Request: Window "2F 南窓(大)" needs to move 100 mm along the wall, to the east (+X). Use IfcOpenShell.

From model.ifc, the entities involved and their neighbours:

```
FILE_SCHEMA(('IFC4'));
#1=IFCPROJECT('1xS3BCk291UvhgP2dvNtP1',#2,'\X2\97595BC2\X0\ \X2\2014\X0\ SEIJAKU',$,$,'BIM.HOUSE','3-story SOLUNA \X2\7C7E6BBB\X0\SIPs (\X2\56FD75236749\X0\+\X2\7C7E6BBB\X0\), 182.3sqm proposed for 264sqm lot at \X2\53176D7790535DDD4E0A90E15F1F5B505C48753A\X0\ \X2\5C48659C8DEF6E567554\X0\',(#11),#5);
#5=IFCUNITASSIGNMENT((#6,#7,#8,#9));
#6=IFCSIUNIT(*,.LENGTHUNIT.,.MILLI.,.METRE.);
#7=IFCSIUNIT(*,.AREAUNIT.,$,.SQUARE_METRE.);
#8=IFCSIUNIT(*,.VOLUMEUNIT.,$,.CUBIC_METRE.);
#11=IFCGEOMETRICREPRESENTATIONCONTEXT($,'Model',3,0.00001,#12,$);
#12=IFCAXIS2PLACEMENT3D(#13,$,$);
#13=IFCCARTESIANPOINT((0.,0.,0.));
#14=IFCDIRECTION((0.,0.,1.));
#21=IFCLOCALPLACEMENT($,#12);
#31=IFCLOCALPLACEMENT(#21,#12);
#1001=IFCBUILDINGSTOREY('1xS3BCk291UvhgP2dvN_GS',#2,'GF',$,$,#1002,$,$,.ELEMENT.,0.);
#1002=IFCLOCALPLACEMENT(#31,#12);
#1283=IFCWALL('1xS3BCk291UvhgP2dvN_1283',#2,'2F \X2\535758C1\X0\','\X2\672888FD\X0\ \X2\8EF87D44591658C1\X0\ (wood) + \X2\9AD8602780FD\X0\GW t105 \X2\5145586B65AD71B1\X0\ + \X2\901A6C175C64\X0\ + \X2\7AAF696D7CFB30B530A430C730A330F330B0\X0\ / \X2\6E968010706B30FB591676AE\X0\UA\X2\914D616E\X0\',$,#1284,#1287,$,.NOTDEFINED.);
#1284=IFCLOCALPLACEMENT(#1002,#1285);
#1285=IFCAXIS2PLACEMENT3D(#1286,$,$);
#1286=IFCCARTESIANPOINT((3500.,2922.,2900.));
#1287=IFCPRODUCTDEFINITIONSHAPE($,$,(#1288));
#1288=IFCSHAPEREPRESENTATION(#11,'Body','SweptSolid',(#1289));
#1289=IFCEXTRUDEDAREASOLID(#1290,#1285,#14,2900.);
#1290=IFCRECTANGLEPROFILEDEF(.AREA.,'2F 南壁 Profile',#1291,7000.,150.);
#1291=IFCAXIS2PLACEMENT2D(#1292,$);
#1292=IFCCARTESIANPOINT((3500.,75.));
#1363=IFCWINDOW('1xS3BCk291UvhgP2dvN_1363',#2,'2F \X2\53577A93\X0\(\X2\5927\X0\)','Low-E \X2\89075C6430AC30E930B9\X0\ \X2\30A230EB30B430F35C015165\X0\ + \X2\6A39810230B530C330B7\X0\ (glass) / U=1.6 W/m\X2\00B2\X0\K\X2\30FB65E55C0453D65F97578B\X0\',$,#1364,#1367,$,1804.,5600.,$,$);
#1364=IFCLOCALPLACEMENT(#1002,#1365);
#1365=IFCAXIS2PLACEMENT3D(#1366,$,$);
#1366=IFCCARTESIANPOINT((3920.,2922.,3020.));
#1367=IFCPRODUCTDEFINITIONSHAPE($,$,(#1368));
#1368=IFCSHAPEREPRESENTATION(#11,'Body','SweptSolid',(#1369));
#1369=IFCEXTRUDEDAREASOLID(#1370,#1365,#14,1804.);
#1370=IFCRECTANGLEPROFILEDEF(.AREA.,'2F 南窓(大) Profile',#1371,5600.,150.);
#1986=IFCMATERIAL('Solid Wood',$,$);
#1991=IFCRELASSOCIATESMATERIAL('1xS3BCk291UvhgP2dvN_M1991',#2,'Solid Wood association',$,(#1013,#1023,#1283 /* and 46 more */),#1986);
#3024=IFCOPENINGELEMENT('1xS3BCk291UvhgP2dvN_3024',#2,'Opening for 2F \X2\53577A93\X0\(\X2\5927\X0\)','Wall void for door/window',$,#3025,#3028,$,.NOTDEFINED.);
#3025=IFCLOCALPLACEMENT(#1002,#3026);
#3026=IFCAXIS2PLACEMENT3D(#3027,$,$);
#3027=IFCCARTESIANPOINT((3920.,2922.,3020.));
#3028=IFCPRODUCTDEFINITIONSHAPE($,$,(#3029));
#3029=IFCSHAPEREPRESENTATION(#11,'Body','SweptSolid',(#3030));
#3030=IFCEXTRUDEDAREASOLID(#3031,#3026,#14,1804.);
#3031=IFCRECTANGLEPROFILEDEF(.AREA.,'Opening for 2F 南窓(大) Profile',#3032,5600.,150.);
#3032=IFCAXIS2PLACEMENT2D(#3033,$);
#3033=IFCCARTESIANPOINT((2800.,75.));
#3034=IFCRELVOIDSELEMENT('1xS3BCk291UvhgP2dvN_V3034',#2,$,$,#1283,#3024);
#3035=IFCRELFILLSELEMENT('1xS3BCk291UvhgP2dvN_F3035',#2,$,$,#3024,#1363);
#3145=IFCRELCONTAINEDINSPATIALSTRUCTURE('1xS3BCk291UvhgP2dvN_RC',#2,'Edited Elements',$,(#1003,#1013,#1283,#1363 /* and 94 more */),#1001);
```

```python
import ifcopenshell
import ifcopenshell.api.geometry
import ifcopenshell.util.placement
import ifcopenshell.util.unit

model = ifcopenshell.open("model.ifc")
unit_scale = ifcopenshell.util.unit.calculate_unit_scale(model)

window = model.by_guid("1xS3BCk291UvhgP2dvN_1363")
opening = window.FillsVoids[0].RelatingOpeningElement
wall = opening.VoidsElements[0].RelatingBuildingElement

wall_matrix = ifcopenshell.util.placement.get_local_placement(wall.ObjectPlacement)
shift = wall_matrix[:3, 0] * 0.1 / unit_scale
before = ifcopenshell.util.placement.get_local_placement(window.ObjectPlacement)[:3, 3].copy()

# The window is not placed relative to its opening, so move both.
for product in (opening, window):
    matrix = ifcopenshell.util.placement.get_local_placement(product.ObjectPlacement)
    matrix[:3, 3] += shift
    ifcopenshell.api.geometry.edit_object_placement(model, product=product, matrix=matrix, is_si=False)

after = ifcopenshell.util.placement.get_local_placement(window.ObjectPlacement)[:3, 3]
print("window moved by", (after - before).round(3) + 0.0)

model.write("model_updated.ifc")
```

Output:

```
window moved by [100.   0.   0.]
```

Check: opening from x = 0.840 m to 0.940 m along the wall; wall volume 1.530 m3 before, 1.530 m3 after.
